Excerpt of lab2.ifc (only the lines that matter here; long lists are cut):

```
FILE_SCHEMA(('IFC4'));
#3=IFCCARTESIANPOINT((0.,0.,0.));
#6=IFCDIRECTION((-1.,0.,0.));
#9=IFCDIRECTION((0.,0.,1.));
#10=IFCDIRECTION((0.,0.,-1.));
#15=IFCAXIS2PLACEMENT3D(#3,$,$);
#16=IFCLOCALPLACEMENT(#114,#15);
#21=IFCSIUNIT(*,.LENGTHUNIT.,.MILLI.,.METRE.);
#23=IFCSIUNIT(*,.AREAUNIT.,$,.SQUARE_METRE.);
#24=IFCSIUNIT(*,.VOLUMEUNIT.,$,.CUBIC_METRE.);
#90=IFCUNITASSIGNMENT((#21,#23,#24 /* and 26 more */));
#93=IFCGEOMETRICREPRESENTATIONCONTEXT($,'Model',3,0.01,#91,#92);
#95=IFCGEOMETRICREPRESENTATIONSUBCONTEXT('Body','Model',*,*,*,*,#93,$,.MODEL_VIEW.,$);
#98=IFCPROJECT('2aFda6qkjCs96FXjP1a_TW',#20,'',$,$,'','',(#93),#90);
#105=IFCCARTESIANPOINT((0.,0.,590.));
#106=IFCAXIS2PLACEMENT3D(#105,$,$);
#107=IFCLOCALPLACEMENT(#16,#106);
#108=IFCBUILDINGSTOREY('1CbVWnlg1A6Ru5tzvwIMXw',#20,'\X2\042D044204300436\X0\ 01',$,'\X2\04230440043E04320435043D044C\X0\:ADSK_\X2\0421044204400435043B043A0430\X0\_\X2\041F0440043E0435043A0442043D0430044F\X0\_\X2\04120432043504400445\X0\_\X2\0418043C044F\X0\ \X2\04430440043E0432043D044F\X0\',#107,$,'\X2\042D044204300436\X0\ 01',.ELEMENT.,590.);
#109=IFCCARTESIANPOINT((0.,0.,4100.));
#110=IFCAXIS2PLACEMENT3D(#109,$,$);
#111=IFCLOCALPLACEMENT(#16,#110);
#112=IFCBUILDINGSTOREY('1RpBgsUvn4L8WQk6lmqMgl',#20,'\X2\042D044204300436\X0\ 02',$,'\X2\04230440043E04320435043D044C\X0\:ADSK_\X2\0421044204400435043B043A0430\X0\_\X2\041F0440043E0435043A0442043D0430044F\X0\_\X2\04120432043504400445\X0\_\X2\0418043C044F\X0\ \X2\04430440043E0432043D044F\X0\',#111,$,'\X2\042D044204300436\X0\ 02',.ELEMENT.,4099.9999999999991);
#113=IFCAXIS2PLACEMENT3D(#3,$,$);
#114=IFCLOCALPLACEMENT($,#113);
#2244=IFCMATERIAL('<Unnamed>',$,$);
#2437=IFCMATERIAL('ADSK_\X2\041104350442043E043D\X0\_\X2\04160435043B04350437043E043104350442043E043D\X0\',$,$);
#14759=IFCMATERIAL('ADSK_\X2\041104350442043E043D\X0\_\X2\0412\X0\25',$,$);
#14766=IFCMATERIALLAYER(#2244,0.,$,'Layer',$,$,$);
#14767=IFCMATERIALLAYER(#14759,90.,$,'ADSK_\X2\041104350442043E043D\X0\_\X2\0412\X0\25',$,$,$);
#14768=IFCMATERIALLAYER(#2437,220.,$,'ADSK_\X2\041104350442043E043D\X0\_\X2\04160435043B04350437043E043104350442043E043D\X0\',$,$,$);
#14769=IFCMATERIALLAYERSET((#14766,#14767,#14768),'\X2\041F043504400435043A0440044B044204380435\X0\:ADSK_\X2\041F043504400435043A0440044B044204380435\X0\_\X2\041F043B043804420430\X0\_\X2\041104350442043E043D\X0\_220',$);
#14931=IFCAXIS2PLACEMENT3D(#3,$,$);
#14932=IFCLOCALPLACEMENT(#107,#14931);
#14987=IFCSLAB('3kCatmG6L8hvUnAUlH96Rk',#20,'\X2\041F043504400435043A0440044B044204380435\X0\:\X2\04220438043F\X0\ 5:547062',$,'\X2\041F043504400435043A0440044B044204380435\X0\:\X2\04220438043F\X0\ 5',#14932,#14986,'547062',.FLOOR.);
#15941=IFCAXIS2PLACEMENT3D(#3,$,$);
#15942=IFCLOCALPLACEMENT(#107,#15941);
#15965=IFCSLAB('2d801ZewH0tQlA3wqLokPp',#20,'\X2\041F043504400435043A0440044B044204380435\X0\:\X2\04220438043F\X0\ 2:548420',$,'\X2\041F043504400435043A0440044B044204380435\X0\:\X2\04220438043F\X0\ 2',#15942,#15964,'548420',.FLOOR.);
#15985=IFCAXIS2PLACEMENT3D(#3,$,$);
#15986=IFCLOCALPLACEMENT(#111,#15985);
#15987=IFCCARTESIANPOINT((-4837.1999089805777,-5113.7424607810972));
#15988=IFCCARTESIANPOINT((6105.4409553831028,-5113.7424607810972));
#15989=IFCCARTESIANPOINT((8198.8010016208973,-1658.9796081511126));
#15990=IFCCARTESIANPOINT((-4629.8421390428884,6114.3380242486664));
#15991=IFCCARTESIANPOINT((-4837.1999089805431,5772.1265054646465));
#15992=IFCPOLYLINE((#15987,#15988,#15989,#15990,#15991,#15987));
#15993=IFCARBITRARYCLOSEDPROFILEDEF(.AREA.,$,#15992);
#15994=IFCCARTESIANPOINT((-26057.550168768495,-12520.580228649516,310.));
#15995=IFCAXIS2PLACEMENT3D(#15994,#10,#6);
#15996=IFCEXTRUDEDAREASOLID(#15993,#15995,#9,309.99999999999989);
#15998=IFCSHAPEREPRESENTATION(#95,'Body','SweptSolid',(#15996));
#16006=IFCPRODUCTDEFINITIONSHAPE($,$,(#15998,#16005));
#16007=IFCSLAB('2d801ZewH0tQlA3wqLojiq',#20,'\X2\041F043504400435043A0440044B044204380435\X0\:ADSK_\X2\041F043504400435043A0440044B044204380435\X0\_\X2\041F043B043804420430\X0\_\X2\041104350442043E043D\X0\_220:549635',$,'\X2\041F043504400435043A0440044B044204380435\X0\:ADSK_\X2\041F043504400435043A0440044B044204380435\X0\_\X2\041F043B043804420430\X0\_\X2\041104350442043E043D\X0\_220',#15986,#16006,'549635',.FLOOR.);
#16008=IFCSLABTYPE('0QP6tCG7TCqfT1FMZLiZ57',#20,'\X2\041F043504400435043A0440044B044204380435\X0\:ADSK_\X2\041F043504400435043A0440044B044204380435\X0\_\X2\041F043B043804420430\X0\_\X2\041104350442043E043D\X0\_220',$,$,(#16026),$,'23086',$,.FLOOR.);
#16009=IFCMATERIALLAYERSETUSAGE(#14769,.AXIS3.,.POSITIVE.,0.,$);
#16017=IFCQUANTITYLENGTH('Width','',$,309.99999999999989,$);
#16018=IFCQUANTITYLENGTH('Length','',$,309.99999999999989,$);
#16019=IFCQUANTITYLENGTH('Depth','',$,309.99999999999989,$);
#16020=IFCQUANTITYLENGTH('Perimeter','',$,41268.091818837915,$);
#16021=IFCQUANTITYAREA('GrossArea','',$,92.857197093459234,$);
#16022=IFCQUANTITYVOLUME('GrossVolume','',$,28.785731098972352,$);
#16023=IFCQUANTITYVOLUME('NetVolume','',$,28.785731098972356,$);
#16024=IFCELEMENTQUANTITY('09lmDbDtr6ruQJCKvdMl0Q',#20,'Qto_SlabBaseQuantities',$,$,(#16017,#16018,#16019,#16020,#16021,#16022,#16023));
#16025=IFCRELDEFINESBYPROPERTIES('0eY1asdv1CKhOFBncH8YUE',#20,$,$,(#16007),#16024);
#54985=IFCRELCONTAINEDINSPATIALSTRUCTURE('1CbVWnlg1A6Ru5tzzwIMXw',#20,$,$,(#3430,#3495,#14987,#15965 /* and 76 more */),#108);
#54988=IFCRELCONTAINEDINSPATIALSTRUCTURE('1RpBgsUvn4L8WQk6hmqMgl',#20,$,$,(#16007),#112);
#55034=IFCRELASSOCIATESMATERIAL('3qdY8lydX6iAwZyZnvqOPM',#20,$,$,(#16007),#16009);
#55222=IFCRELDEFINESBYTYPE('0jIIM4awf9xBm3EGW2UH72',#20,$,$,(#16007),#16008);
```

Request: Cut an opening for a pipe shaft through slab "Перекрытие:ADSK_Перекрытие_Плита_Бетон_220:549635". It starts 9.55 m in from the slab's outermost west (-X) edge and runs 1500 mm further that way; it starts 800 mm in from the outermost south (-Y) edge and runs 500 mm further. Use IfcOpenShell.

```python
import numpy as np
import ifcopenshell
import ifcopenshell.api.feature
import ifcopenshell.api.geometry
import ifcopenshell.api.pset
import ifcopenshell.api.root
import ifcopenshell.geom
import ifcopenshell.util.element
import ifcopenshell.util.placement
import ifcopenshell.util.representation
import ifcopenshell.util.shape
import ifcopenshell.util.unit

model = ifcopenshell.open("lab2.ifc")
unit_scale = ifcopenshell.util.unit.calculate_unit_scale(model)
volume_scale = ifcopenshell.util.unit.calculate_unit_scale(model, "VOLUMEUNIT")
settings = ifcopenshell.geom.settings()


def volume(element):
    """Net volume in cubic metres, openings subtracted."""
    shape = ifcopenshell.geom.create_shape(settings, element)
    return ifcopenshell.util.shape.get_volume(shape.geometry)


slab = model.by_guid("2d801ZewH0tQlA3wqLojiq")
before = volume(slab)

# Extent in the slab's own axes, in metres. The edges named are its -X and -Y sides.
slab_shape = ifcopenshell.geom.create_shape(settings, slab)
vertices = ifcopenshell.util.shape.get_vertices(slab_shape.geometry)
x_min, y_min, bottom = vertices.min(axis=0)
top = vertices[:, 2].max()

opening = ifcopenshell.api.root.create_entity(model, ifc_class="IfcOpeningElement", name="Pipe shaft opening", predefined_type="OPENING")
context = ifcopenshell.util.representation.get_context(model, "Model", "Body", "MODEL_VIEW")
width, depth = 1.5, 0.5
outline = [(0.0, 0.0), (width, 0.0), (width, depth), (0.0, depth), (0.0, 0.0)]
# Overshoot both faces by 50 mm so the cut is clean.
shape = ifcopenshell.api.geometry.add_slab_representation(
    model, context=context, depth=top - bottom + 0.1, polyline=outline
)
ifcopenshell.api.geometry.assign_representation(model, product=opening, representation=shape)

matrix = ifcopenshell.util.placement.get_local_placement(slab.ObjectPlacement)
matrix[:, 3] = matrix @ np.append(np.array([x_min + 9.55, y_min + 0.8, bottom - 0.05]) / unit_scale, 1.0)
ifcopenshell.api.geometry.edit_object_placement(model, product=opening, matrix=matrix, is_si=False)
ifcopenshell.api.feature.add_feature(model, feature=opening, element=slab)

after = volume(slab)

# Update the slab's stored quantities.
qto = model.by_id(ifcopenshell.util.element.get_pset(slab, "Qto_SlabBaseQuantities", should_inherit=False)["id"])
ifcopenshell.api.pset.edit_qto(model, qto=qto, properties={"NetVolume": after / volume_scale})

print(f"slab volume {before:.3f} -> {after:.3f} m3")

model.write("lab2_v2.ifc")
```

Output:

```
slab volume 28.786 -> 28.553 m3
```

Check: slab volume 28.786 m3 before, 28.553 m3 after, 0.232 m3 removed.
